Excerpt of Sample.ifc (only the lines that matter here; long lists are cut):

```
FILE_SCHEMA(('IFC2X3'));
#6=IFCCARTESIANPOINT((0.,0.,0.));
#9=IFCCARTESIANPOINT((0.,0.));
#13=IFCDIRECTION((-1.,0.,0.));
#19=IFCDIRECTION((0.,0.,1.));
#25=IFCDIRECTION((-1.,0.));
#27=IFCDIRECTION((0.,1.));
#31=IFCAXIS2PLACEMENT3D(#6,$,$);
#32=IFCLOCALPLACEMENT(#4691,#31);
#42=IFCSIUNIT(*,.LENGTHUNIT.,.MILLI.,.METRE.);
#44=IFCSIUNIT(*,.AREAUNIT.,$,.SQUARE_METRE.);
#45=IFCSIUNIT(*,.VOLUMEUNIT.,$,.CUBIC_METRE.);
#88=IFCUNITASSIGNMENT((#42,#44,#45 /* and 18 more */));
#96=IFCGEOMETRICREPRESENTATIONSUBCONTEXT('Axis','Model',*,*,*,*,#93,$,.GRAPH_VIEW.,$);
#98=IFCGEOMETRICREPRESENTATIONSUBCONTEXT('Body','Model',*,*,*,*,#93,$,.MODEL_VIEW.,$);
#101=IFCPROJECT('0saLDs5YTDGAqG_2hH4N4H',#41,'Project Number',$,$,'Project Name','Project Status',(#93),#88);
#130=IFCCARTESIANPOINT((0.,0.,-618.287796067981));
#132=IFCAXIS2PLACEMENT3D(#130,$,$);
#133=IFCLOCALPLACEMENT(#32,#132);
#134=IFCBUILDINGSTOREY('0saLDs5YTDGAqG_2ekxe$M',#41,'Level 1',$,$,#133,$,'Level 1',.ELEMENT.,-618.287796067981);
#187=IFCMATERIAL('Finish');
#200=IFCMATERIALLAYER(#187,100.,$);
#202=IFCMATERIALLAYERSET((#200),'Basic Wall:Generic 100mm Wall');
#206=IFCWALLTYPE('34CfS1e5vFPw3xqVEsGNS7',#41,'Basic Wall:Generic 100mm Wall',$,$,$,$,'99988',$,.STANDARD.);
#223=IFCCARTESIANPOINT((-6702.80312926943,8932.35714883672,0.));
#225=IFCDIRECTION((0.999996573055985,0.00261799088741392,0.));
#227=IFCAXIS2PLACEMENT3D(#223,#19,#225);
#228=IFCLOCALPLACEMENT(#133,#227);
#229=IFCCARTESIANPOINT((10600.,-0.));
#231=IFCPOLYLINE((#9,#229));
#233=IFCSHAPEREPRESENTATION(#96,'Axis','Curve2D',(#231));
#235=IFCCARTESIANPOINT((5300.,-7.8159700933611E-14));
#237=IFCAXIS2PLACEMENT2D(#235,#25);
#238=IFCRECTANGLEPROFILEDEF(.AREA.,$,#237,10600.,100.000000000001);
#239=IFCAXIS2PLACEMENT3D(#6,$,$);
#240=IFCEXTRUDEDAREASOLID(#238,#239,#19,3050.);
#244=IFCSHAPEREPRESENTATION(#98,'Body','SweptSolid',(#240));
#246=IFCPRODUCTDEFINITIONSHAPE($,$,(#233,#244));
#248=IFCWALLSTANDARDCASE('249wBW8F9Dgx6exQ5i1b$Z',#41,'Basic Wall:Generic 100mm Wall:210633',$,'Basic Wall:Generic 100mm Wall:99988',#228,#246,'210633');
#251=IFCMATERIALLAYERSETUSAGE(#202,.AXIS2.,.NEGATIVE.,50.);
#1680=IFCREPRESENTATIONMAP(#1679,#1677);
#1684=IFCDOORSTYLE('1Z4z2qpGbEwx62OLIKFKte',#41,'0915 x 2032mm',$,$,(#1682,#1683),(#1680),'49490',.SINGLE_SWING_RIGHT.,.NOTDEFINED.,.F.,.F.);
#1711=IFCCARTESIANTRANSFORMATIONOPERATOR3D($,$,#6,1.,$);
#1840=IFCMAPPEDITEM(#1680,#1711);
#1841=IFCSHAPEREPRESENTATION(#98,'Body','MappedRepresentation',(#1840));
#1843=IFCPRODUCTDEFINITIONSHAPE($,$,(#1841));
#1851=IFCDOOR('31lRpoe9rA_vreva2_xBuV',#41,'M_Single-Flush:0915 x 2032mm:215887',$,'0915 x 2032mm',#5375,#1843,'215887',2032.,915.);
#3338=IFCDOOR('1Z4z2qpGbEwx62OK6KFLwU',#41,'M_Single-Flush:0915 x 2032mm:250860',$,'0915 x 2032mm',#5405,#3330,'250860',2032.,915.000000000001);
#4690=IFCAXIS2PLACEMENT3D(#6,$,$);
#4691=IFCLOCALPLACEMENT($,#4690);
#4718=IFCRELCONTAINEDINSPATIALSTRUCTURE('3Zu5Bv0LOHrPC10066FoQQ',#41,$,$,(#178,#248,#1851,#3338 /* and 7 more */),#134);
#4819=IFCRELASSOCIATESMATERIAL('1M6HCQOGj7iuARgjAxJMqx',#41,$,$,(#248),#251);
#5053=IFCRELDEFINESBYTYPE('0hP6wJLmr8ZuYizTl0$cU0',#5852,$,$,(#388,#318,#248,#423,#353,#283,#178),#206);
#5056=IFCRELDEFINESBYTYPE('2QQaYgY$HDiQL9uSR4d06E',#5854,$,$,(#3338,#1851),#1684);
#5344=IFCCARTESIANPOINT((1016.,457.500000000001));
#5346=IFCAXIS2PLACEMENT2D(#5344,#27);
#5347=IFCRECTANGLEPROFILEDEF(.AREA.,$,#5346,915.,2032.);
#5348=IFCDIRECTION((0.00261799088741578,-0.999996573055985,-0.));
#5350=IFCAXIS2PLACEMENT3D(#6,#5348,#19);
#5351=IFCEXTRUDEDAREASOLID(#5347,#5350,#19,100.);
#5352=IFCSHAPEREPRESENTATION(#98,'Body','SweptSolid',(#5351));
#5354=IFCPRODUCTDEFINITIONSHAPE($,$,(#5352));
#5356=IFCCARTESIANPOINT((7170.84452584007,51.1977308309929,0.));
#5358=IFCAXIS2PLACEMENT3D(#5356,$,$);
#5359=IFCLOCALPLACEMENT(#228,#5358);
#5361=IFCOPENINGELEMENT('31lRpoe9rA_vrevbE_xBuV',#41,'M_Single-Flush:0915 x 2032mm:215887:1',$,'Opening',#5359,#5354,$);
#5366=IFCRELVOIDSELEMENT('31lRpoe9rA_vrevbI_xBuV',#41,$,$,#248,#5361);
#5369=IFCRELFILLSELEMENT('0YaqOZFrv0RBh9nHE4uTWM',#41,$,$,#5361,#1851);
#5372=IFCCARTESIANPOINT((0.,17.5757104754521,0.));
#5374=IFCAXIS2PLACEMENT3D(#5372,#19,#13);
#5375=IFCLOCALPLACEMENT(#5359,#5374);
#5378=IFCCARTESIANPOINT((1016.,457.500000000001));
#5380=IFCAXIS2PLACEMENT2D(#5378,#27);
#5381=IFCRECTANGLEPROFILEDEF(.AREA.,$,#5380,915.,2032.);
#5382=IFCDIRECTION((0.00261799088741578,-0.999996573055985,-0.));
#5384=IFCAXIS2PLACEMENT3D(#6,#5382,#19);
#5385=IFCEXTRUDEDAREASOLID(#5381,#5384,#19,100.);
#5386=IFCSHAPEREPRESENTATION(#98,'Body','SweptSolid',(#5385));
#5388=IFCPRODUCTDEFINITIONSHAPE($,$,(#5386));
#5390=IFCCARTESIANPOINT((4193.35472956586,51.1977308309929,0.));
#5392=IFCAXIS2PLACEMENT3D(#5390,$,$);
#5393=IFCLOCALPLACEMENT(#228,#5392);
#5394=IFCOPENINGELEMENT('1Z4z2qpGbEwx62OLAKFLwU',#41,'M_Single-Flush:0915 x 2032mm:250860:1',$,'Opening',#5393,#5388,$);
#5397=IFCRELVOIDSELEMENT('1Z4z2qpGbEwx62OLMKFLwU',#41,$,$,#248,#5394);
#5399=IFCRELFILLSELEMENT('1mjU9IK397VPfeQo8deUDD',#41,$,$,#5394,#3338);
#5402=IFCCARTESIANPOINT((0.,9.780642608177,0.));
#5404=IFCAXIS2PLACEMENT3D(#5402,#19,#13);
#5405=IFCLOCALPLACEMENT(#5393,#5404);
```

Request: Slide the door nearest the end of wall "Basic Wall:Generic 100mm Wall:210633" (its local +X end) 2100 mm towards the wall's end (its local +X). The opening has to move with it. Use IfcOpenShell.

```python
import ifcopenshell
import ifcopenshell.api.geometry
import ifcopenshell.util.placement

model = ifcopenshell.open("Sample.ifc")

door = model.by_id(1851)
opening = door.FillsVoids[0].RelatingOpeningElement
wall = opening.VoidsElements[0].RelatingBuildingElement

wall_matrix = ifcopenshell.util.placement.get_local_placement(wall.ObjectPlacement)
shift = wall_matrix[:3, 0] * 2100.0
before = ifcopenshell.util.placement.get_local_placement(door.ObjectPlacement)[:3, 3].copy()

# The door is placed relative to its opening, so it follows when the opening moves.
matrix = ifcopenshell.util.placement.get_local_placement(opening.ObjectPlacement)
matrix[:3, 3] += shift
ifcopenshell.api.geometry.edit_object_placement(
    model, product=opening, matrix=matrix, is_si=False, should_transform_children=True
)

after = ifcopenshell.util.placement.get_local_placement(door.ObjectPlacement)[:3, 3]
print("door moved by", (after - before).round(3) + 0.0)

model.write("Sample_edited.ifc")
```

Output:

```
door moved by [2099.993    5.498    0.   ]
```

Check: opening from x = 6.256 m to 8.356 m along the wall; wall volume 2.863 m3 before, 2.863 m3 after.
